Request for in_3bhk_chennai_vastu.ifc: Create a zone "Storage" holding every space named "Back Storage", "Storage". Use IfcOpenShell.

First a look at what the model holds.

```python
import ifcopenshell

model = ifcopenshell.open("in_3bhk_chennai_vastu.ifc")
print(model.schema)
seen = {}
for space in model.by_type("IfcSpace"):
    seen[space.LongName] = seen.get(space.LongName, 0) + 1
for name, count in sorted(seen.items(), key=str):
    print(count, "x", name)
print("zones:", [z.Name for z in model.by_type("IfcZone")][:20])
```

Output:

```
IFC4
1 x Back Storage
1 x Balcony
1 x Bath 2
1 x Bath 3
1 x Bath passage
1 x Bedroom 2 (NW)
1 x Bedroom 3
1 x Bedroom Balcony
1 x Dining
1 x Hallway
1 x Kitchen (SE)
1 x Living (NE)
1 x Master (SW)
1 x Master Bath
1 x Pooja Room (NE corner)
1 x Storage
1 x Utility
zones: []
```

```python
import ifcopenshell
import ifcopenshell.api.group
import ifcopenshell.api.root

model = ifcopenshell.open("in_3bhk_chennai_vastu.ifc")

names = {"Back Storage", "Storage"}
spaces = [s for s in model.by_type("IfcSpace") if s.LongName in names]

zone = ifcopenshell.api.root.create_entity(model, ifc_class="IfcZone", name="Storage")
ifcopenshell.api.group.assign_group(model, products=spaces, group=zone)
print(len(spaces), "spaces in", zone.Name)

model.write("in_3bhk_chennai_vastu_edited.ifc")
```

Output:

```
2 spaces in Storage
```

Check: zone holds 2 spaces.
